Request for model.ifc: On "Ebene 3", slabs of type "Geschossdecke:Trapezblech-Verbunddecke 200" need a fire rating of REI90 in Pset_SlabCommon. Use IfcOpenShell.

First a look at what the model holds.

```python
import ifcopenshell
import ifcopenshell.util.element

model = ifcopenshell.open("model.ifc")
print(model.schema)
storey = next(s for s in model.by_type("IfcBuildingStorey") if s.Name == "Ebene 3")
slabs = [e for e in ifcopenshell.util.element.get_decomposition(storey) if e.is_a("IfcSlab")]
seen = {}
for e in slabs:
    element_type = ifcopenshell.util.element.get_type(e)
    key = (element_type.Name if element_type != e and element_type else None, ifcopenshell.util.element.get_pset(e, "Pset_SlabCommon", "FireRating"))
    seen[key] = seen.get(key, 0) + 1
for (name, value), count in sorted(seen.items(), key=str):
    print(count, "x", name, "|", value)
```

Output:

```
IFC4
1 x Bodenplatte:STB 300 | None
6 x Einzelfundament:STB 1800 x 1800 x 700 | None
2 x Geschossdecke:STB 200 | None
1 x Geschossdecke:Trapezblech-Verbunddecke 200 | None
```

```python
import ifcopenshell
import ifcopenshell.api.pset
import ifcopenshell.util.element

model = ifcopenshell.open("model.ifc")

storey = next(s for s in model.by_type("IfcBuildingStorey") if s.Name == "Ebene 3")
slabs = [e for e in ifcopenshell.util.element.get_decomposition(storey) if e.is_a("IfcSlab")]

count = 0
for e in slabs:
    element_type = ifcopenshell.util.element.get_type(e)
    if element_type in (None, e) or element_type.Name != "Geschossdecke:Trapezblech-Verbunddecke 200":
        continue
    # add_pset returns the element's existing set when there is one.
    pset = ifcopenshell.api.pset.add_pset(model, product=e, name="Pset_SlabCommon")
    ifcopenshell.api.pset.edit_pset(model, pset=pset, properties={"FireRating": "REI90"})
    count += 1

print(count, "slabs updated")

model.write("model_updated.ifc")
```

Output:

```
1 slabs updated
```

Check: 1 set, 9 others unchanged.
